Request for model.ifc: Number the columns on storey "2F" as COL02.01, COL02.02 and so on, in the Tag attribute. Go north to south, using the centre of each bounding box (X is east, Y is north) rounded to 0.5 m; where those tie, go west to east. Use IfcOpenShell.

First a look at what the model holds.

```python
import ifcopenshell
import ifcopenshell.util.element
import ifcopenshell.util.placement

model = ifcopenshell.open("model.ifc")
print(model.schema)
storey = next(s for s in model.by_type("IfcBuildingStorey") if s.Name == "2F")
columns = [e for e in ifcopenshell.util.element.get_decomposition(storey) if e.is_a("IfcColumn")]
for e in sorted(columns, key=lambda e: e.id()):
    origin = ifcopenshell.util.placement.get_local_placement(e.ObjectPlacement)[:3, 3]
    print(e.id(), e.Tag, e.Name, origin.round(2) + 0.0, sep=" | ")
```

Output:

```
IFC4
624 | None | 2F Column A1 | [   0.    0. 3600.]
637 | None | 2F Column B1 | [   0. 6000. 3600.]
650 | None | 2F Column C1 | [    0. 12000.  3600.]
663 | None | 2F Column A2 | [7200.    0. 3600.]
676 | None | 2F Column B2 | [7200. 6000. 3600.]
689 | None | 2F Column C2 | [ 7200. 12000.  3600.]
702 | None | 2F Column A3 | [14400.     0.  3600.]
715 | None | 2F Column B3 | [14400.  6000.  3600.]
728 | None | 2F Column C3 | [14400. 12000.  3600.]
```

```python
import ifcopenshell
import ifcopenshell.geom
import ifcopenshell.util.element
import ifcopenshell.util.shape

model = ifcopenshell.open("model.ifc")
settings = ifcopenshell.geom.settings()
settings.set("use-world-coords", True)


def centre(element):
    shape = ifcopenshell.geom.create_shape(settings, element)
    return ifcopenshell.util.shape.get_bbox_centroid(shape.geometry)


storey = next(s for s in model.by_type("IfcBuildingStorey") if s.Name == "2F")
columns = [e for e in ifcopenshell.util.element.get_decomposition(storey) if e.is_a("IfcColumn")]

# Insertion points can sit at a corner or the storey origin, so sort by the geometry (in metres).
centres = {e: centre(e) for e in columns}
columns.sort(key=lambda e: (-round(centres[e][1] / 0.5), centres[e][0]))

for i, e in enumerate(columns, start=1):
    number = f"COL02.{i:02d}"
    e.Tag = number
    print(e.id(), number)

model.write("model_v2.ifc")
```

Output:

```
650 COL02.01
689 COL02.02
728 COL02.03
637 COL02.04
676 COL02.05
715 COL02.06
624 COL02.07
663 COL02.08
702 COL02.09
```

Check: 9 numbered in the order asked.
